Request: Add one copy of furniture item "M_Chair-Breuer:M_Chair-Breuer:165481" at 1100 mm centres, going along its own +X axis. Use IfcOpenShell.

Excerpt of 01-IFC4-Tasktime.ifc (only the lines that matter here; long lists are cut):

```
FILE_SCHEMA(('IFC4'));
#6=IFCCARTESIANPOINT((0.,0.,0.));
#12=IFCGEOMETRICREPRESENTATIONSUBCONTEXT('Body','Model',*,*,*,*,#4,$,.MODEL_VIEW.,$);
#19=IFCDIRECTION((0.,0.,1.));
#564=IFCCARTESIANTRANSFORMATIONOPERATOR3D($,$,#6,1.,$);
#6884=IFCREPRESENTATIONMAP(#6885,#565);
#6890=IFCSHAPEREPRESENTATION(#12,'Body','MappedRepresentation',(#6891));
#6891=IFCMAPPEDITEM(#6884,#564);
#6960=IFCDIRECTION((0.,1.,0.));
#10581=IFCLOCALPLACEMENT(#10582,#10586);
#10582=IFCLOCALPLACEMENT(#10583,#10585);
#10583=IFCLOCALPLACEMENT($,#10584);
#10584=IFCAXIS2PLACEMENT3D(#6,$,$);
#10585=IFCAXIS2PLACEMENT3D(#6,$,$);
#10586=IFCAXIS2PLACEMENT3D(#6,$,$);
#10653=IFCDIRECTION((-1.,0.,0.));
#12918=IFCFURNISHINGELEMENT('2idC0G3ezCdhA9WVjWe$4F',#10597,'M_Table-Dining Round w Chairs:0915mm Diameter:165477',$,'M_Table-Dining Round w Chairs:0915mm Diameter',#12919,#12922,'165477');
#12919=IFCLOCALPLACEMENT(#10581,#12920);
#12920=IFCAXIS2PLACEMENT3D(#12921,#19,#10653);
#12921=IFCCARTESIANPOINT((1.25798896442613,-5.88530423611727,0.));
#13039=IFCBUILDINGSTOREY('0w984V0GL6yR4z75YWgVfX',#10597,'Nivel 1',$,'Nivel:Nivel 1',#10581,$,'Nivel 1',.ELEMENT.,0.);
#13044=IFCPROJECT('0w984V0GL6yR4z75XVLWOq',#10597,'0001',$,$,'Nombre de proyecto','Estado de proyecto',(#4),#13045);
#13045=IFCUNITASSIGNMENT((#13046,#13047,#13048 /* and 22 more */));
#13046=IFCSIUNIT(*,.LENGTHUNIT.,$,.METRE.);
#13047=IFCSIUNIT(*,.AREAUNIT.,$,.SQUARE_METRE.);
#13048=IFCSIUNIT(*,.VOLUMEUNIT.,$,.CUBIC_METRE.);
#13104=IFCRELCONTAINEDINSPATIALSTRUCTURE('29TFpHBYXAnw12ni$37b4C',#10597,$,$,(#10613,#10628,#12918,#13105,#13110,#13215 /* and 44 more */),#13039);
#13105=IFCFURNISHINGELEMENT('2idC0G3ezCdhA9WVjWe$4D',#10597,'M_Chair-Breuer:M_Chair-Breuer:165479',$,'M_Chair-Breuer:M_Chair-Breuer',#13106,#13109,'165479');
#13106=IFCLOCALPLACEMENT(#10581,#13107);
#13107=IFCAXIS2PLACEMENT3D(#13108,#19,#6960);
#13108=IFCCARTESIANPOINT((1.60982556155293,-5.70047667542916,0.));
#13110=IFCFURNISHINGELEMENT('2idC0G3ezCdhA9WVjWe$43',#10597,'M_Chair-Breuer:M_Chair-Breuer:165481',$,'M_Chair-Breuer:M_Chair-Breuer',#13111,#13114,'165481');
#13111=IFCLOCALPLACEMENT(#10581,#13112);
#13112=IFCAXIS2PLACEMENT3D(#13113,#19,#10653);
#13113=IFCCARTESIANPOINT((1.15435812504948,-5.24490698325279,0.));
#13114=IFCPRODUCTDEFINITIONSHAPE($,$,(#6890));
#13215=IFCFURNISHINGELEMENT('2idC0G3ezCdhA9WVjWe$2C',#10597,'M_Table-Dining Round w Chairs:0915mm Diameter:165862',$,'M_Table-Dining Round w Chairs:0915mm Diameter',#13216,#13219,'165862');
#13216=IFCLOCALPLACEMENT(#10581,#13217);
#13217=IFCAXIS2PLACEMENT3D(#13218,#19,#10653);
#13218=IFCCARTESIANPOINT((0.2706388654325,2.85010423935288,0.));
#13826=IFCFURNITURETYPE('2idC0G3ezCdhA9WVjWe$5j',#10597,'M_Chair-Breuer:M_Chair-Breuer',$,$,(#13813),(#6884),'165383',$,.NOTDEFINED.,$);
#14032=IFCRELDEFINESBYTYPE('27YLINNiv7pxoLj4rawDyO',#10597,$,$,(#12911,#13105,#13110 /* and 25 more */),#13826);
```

```python
import ifcopenshell
import ifcopenshell.api.geometry
import ifcopenshell.api.root
import ifcopenshell.util.element
import ifcopenshell.util.placement

model = ifcopenshell.open("01-IFC4-Tasktime.ifc")


def reuse_history(source, copy):
    """copy_class also copies each property set's owner history, people and application; keep the originals."""
    for rel in copy.IsDefinedBy:
        if rel.is_a("IfcRelDefinesByProperties") and (history := rel.RelatingPropertyDefinition.OwnerHistory):
            rel.RelatingPropertyDefinition.OwnerHistory = source.OwnerHistory
            ifcopenshell.util.element.remove_deep2(model, history)


source = model.by_guid("2idC0G3ezCdhA9WVjWe$43")
base = ifcopenshell.util.placement.get_local_placement(source.ObjectPlacement)
step = base[:3, 0] * 1.1

for i in range(1, 2):
    copy = ifcopenshell.api.root.copy_class(model, product=source)
    copy.Representation = ifcopenshell.util.element.copy_deep(
        model, source.Representation, exclude=["IfcGeometricRepresentationContext", "IfcRepresentationMap"]
    )
    copy.Name = "M_Chair-Breuer:M_Chair-Breuer"
    copy.Tag = None
    reuse_history(source, copy)
    matrix = base.copy()
    matrix[:3, 3] += i * step
    print("added at", matrix[:3, 3].round(3) + 0.0)
    ifcopenshell.api.geometry.edit_object_placement(model, product=copy, matrix=matrix, is_si=False)

model.write("01-IFC4-Tasktime_edited.ifc")
```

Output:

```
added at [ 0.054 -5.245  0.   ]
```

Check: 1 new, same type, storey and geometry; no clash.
